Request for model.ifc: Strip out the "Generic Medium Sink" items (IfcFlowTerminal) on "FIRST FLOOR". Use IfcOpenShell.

First a look at what the model holds.

```python
import ifcopenshell
import ifcopenshell.util.element

model = ifcopenshell.open("model.ifc")
print(model.schema)
storey = next(s for s in model.by_type("IfcBuildingStorey") if s.Name == "FIRST FLOOR")
terminals = [e for e in ifcopenshell.util.element.get_decomposition(storey) if e.is_a("IfcFlowTerminal")]
seen = {}
for e in terminals:
    element_type = ifcopenshell.util.element.get_type(e)
    name = element_type.Name if element_type not in (None, e) else None
    seen[name] = seen.get(name, 0) + 1
for name, count in sorted(seen.items(), key=str):
    print(count, "x", name)
```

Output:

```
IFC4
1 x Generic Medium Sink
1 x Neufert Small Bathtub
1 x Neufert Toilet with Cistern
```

```python
import ifcopenshell
import ifcopenshell.api.root
import ifcopenshell.util.element

model = ifcopenshell.open("model.ifc")

storey = next(s for s in model.by_type("IfcBuildingStorey") if s.Name == "FIRST FLOOR")
terminals = [e for e in ifcopenshell.util.element.get_decomposition(storey) if e.is_a("IfcFlowTerminal")]
targets = [e for e in terminals if (t := ifcopenshell.util.element.get_type(e)) not in (None, e) and t.Name == "Generic Medium Sink"]

for e in targets:
    ifcopenshell.api.root.remove_product(model, product=e)
print(len(targets), "removed")

model.write("model_updated.ifc")
```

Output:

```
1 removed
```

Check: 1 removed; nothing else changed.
